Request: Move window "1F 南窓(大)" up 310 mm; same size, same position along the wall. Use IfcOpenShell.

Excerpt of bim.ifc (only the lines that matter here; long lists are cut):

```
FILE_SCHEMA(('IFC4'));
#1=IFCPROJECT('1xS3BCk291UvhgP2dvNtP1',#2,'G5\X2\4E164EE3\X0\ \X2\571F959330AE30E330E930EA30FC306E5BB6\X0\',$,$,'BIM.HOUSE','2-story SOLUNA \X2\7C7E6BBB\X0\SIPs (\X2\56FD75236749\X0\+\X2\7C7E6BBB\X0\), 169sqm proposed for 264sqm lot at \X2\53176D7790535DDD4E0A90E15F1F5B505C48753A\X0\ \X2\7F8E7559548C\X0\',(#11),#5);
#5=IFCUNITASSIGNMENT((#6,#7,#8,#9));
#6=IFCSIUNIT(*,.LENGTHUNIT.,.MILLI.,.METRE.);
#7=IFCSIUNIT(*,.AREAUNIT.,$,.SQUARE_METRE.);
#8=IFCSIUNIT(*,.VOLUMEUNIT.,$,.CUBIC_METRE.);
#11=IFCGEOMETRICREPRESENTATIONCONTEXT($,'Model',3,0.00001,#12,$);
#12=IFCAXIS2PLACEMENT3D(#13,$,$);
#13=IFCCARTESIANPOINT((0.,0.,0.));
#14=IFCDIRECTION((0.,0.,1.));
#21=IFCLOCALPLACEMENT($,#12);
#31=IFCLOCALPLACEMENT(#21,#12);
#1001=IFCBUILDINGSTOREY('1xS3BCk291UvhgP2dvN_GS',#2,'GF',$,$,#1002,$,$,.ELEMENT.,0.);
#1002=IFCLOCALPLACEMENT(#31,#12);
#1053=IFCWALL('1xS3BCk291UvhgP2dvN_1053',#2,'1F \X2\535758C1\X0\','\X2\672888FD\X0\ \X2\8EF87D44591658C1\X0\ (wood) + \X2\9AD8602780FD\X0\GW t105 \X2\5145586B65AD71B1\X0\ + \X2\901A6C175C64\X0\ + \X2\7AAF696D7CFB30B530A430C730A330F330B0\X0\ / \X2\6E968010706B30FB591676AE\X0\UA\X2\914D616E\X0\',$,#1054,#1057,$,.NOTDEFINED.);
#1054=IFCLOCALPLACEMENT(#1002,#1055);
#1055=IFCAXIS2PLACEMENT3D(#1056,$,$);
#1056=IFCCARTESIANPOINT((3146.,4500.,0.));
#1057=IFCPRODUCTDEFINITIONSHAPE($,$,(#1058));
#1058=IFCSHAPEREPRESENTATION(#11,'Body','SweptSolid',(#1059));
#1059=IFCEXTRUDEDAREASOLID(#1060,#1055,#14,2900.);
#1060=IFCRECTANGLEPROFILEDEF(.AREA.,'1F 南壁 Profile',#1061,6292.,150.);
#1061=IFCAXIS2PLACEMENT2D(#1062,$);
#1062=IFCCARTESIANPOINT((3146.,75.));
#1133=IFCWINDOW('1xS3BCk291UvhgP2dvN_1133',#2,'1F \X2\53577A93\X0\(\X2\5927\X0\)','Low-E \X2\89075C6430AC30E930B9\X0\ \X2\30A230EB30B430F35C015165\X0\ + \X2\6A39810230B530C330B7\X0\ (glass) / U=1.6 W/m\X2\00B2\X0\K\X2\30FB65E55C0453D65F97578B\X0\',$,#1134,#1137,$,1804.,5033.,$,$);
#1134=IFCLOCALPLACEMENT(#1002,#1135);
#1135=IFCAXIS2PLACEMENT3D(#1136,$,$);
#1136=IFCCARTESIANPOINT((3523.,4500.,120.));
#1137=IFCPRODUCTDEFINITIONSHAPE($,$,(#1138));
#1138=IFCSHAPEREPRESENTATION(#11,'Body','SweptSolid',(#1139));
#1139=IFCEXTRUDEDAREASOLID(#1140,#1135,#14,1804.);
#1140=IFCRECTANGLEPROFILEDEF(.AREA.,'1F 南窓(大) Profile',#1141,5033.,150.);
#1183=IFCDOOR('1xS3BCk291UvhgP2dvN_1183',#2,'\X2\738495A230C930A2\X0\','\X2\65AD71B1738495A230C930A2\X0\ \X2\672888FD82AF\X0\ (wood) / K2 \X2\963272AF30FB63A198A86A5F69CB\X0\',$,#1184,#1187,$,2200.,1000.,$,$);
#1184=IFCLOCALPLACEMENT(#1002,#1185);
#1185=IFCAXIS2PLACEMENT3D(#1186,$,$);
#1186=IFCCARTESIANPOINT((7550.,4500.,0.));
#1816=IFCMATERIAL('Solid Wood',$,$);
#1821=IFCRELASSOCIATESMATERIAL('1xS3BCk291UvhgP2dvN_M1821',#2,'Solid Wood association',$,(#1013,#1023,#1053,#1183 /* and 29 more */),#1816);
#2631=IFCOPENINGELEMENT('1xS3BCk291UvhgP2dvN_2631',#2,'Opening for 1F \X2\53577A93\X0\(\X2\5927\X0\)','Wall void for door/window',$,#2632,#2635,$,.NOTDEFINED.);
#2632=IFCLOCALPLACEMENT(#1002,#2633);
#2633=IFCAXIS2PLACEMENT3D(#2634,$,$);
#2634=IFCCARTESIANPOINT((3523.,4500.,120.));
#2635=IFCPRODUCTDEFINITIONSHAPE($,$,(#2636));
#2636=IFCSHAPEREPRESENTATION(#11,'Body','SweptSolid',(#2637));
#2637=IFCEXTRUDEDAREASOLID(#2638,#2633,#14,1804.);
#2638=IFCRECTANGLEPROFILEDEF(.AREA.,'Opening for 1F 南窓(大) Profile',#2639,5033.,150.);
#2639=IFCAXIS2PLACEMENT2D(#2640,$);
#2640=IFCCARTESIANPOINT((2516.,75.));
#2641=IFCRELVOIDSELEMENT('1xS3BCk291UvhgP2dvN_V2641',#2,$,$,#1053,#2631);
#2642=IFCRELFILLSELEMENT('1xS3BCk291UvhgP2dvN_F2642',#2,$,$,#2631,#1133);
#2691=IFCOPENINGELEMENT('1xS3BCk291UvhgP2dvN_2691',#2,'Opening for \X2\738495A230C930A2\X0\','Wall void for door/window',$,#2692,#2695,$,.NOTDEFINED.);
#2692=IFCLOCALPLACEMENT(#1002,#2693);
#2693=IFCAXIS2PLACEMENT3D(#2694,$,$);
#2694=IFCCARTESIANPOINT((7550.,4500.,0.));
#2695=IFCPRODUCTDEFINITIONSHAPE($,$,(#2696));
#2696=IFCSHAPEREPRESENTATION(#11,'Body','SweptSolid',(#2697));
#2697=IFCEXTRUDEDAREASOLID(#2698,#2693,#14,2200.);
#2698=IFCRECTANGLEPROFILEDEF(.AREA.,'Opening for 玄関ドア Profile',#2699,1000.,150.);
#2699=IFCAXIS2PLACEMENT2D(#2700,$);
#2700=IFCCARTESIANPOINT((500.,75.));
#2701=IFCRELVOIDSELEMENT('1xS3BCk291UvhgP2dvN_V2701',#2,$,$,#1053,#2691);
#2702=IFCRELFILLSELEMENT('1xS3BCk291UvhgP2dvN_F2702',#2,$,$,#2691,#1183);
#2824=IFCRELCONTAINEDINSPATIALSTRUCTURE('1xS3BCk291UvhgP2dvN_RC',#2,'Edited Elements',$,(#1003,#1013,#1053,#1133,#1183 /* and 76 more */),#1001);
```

```python
import numpy as np
import ifcopenshell
import ifcopenshell.api.geometry
import ifcopenshell.util.placement
import ifcopenshell.util.unit

model = ifcopenshell.open("bim.ifc")
unit_scale = ifcopenshell.util.unit.calculate_unit_scale(model)

window = model.by_guid("1xS3BCk291UvhgP2dvN_1133")
opening = window.FillsVoids[0].RelatingOpeningElement
dz = 0.31 / unit_scale

shift = np.array([0.0, 0.0, dz])
# The window is not placed relative to its opening, so move both.
for product in (opening, window):
    matrix = ifcopenshell.util.placement.get_local_placement(product.ObjectPlacement)
    matrix[:3, 3] += shift
    ifcopenshell.api.geometry.edit_object_placement(model, product=product, matrix=matrix, is_si=False)

print(f"moved by {dz * unit_scale:+.3f} m")

model.write("bim-out.ifc")
```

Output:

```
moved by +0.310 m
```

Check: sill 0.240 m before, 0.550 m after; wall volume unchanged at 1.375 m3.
